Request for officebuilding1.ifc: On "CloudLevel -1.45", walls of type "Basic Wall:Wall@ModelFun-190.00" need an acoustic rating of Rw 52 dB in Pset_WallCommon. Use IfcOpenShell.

First a look at what the model holds.

```python
import ifcopenshell
import ifcopenshell.util.element

model = ifcopenshell.open("officebuilding1.ifc")
print(model.schema)
storey = next(s for s in model.by_type("IfcBuildingStorey") if s.Name == "CloudLevel -1.45")
walls = [e for e in ifcopenshell.util.element.get_decomposition(storey) if e.is_a("IfcWall")]
seen = {}
for e in walls:
    element_type = ifcopenshell.util.element.get_type(e)
    key = (element_type.Name if element_type != e and element_type else None, ifcopenshell.util.element.get_pset(e, "Pset_WallCommon", "AcousticRating"))
    seen[key] = seen.get(key, 0) + 1
for (name, value), count in sorted(seen.items(), key=str):
    print(count, "x", name, "|", value)
```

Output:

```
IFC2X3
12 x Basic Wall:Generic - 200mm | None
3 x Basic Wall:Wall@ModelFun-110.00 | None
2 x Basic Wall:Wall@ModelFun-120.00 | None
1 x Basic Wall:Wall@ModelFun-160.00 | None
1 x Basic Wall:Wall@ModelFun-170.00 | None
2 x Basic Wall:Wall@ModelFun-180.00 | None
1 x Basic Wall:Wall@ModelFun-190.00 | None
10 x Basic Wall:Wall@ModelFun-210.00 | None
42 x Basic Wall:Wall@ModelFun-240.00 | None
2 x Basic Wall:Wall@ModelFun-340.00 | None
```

```python
import ifcopenshell
import ifcopenshell.api.pset
import ifcopenshell.util.element

model = ifcopenshell.open("officebuilding1.ifc")

storey = next(s for s in model.by_type("IfcBuildingStorey") if s.Name == "CloudLevel -1.45")
walls = [e for e in ifcopenshell.util.element.get_decomposition(storey) if e.is_a("IfcWall")]

count = 0
for e in walls:
    element_type = ifcopenshell.util.element.get_type(e)
    if element_type in (None, e) or element_type.Name != "Basic Wall:Wall@ModelFun-190.00":
        continue
    # add_pset returns the element's existing set when there is one.
    pset = ifcopenshell.api.pset.add_pset(model, product=e, name="Pset_WallCommon")
    ifcopenshell.api.pset.edit_pset(model, pset=pset, properties={"AcousticRating": "Rw 52 dB"})
    count += 1

print(count, "walls updated")

model.write("officebuilding1-out.ifc")
```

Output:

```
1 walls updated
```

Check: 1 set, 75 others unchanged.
